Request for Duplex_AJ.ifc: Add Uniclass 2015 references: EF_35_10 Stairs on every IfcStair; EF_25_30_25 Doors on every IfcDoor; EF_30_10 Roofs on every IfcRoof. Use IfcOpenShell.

First a look at what the model holds.

```python
import ifcopenshell

model = ifcopenshell.open("Duplex_AJ.ifc")
print(model.schema)
print("classifications:", [c.Name for c in model.by_type("IfcClassification")])
for ifc_class in ("IfcDoor", "IfcRoof", "IfcStair", "IfcWall", "IfcWindow"):
    print(ifc_class, len(model.by_type(ifc_class)))
```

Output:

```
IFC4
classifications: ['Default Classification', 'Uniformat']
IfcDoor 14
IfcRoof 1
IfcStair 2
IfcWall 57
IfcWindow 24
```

```python
import ifcopenshell
import ifcopenshell.api.classification

model = ifcopenshell.open("Duplex_AJ.ifc")

system = ifcopenshell.api.classification.add_classification(model, classification="Uniclass 2015")

codes = {
    "IfcStair": ("EF_35_10", "Stairs"),
    "IfcDoor": ("EF_25_30_25", "Doors"),
    "IfcRoof": ("EF_30_10", "Roofs"),
}
for ifc_class, (code, name) in codes.items():
    products = model.by_type(ifc_class)
    ifcopenshell.api.classification.add_reference(
        model, products=products, classification=system, identification=code, name=name
    )
    print(code, len(products))

model.write("Duplex_AJ_updated.ifc")
```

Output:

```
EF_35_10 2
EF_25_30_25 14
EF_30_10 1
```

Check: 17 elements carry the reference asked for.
